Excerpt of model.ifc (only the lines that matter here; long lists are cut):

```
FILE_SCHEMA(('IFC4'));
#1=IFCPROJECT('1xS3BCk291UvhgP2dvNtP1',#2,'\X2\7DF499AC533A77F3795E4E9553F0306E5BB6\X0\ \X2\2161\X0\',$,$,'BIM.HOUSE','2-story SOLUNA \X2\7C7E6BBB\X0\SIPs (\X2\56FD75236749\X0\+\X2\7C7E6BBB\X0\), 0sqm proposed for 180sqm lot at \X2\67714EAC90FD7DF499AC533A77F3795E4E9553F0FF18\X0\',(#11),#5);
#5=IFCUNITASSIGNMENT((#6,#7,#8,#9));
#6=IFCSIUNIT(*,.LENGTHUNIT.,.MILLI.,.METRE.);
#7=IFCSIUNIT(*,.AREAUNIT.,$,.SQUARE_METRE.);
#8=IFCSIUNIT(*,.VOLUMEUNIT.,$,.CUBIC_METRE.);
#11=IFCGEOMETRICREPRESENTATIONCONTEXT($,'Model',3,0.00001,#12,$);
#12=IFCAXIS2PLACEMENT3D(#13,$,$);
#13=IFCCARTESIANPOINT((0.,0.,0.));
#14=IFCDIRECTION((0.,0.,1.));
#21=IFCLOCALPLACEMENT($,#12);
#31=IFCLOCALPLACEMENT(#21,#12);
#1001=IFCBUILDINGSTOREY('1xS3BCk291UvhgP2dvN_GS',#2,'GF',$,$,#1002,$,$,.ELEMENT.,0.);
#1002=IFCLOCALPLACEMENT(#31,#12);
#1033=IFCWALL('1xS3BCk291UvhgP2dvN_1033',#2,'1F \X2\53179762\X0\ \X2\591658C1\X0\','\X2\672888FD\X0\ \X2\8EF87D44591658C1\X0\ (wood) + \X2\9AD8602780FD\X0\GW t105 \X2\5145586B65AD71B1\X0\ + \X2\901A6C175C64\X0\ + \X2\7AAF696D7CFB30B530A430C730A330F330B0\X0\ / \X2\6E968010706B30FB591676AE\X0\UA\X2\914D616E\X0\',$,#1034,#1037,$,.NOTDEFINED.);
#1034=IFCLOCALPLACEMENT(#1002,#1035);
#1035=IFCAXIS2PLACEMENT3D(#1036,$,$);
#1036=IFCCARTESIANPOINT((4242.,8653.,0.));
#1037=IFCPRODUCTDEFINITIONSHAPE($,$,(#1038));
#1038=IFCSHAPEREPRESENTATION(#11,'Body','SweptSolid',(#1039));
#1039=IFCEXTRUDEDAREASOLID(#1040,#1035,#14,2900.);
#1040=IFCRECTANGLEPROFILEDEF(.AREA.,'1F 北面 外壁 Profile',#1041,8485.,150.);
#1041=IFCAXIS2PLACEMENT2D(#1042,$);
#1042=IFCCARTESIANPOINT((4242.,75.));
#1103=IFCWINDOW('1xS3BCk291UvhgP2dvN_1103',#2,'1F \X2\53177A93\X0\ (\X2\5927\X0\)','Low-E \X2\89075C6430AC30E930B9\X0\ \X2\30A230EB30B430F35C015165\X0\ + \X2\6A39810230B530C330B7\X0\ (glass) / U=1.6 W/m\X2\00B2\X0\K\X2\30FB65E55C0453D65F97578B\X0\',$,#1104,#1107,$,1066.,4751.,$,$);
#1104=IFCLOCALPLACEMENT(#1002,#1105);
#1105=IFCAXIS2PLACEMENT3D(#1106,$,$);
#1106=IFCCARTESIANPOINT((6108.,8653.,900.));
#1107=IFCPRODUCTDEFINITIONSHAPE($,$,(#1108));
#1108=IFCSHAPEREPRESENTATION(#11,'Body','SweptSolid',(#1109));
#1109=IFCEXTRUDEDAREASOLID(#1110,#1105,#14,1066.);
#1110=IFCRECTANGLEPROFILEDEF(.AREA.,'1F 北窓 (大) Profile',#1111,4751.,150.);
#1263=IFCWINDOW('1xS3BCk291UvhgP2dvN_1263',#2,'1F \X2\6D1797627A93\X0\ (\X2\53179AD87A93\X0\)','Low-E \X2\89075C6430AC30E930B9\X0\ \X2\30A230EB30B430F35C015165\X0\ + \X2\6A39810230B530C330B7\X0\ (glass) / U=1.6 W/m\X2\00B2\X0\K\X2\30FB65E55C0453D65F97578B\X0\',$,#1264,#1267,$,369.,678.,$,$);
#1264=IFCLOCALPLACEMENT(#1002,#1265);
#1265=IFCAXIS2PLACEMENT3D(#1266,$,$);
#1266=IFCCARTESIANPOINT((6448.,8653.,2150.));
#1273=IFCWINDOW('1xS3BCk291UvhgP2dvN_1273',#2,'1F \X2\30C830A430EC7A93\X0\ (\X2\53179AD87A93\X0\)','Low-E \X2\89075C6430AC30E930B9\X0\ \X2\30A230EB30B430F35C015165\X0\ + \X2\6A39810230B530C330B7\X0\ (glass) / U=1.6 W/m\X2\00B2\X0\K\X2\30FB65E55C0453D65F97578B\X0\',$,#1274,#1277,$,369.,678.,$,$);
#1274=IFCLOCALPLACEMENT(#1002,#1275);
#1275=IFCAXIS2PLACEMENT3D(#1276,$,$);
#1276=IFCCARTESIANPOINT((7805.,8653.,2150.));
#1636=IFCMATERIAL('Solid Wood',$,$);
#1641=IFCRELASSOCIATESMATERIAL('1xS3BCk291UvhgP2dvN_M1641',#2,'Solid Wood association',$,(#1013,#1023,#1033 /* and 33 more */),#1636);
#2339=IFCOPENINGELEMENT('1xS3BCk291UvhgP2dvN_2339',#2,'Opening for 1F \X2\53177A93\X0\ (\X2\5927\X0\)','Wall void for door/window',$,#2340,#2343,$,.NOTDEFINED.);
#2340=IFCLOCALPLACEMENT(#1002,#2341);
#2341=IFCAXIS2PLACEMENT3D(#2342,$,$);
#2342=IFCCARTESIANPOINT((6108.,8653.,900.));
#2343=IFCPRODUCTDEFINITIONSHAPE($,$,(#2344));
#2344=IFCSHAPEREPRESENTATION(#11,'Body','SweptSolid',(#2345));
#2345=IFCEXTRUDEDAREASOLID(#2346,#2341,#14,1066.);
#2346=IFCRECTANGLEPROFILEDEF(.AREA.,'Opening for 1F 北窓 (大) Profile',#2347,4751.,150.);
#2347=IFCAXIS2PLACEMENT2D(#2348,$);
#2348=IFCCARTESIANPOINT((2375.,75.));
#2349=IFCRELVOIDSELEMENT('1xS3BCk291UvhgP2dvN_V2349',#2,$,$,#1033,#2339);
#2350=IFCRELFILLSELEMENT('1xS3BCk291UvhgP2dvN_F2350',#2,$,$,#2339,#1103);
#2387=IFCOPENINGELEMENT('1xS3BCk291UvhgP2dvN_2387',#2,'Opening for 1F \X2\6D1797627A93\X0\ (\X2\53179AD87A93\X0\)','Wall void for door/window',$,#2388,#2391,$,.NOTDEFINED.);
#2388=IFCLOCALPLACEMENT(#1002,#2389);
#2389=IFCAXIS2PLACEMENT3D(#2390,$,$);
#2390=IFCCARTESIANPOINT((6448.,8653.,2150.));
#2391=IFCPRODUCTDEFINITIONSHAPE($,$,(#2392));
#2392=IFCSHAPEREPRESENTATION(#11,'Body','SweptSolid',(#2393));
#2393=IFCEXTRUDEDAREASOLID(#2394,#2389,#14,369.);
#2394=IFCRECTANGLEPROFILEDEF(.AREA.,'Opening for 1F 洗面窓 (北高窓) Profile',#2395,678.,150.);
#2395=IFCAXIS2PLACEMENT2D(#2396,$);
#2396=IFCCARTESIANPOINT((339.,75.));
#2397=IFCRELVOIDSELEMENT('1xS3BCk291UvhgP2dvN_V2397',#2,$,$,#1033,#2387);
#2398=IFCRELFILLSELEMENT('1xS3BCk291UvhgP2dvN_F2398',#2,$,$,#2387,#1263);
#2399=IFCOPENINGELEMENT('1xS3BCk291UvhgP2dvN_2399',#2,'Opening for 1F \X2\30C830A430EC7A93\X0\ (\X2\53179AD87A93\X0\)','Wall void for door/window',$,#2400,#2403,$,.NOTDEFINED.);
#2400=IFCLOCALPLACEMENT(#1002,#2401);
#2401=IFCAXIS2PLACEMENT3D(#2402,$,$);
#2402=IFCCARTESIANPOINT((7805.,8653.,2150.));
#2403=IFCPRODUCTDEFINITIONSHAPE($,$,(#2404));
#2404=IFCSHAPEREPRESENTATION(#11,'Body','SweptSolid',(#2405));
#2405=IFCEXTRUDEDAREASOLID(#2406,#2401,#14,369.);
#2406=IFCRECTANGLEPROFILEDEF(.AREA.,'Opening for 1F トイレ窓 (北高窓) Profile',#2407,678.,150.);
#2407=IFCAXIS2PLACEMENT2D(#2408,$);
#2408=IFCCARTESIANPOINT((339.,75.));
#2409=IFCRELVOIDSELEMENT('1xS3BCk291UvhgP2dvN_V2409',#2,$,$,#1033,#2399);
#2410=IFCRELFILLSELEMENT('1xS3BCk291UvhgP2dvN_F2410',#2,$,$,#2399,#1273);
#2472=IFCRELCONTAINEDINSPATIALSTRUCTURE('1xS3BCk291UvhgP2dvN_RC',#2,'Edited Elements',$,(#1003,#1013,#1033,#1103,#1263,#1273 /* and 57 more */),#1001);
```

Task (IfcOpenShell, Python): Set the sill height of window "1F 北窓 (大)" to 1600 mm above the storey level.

```python
import numpy as np
import ifcopenshell
import ifcopenshell.api.geometry
import ifcopenshell.geom
import ifcopenshell.util.element
import ifcopenshell.util.placement
import ifcopenshell.util.shape
import ifcopenshell.util.unit

model = ifcopenshell.open("model.ifc")
unit_scale = ifcopenshell.util.unit.calculate_unit_scale(model)

window = model.by_guid("1xS3BCk291UvhgP2dvN_1103")
opening = window.FillsVoids[0].RelatingOpeningElement
storey = ifcopenshell.util.element.get_container(window, ifc_class="IfcBuildingStorey")
level = ifcopenshell.util.placement.get_local_placement(storey.ObjectPlacement)[2, 3]

# The opening's origin need not be at the sill, so measure its lowest point.
shape = ifcopenshell.geom.create_shape(ifcopenshell.geom.settings(), opening)
bottom = ifcopenshell.util.shape.get_shape_bottom_elevation(shape, shape.geometry) / unit_scale
dz = level + 1600.0 - bottom

shift = np.array([0.0, 0.0, dz])
# The window is not placed relative to its opening, so move both.
for product in (opening, window):
    matrix = ifcopenshell.util.placement.get_local_placement(product.ObjectPlacement)
    matrix[:3, 3] += shift
    ifcopenshell.api.geometry.edit_object_placement(model, product=product, matrix=matrix, is_si=False)

print(f"moved by {dz * unit_scale:+.3f} m")

model.write("model_v2.ifc")
```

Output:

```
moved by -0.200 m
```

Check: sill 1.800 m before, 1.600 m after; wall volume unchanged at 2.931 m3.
